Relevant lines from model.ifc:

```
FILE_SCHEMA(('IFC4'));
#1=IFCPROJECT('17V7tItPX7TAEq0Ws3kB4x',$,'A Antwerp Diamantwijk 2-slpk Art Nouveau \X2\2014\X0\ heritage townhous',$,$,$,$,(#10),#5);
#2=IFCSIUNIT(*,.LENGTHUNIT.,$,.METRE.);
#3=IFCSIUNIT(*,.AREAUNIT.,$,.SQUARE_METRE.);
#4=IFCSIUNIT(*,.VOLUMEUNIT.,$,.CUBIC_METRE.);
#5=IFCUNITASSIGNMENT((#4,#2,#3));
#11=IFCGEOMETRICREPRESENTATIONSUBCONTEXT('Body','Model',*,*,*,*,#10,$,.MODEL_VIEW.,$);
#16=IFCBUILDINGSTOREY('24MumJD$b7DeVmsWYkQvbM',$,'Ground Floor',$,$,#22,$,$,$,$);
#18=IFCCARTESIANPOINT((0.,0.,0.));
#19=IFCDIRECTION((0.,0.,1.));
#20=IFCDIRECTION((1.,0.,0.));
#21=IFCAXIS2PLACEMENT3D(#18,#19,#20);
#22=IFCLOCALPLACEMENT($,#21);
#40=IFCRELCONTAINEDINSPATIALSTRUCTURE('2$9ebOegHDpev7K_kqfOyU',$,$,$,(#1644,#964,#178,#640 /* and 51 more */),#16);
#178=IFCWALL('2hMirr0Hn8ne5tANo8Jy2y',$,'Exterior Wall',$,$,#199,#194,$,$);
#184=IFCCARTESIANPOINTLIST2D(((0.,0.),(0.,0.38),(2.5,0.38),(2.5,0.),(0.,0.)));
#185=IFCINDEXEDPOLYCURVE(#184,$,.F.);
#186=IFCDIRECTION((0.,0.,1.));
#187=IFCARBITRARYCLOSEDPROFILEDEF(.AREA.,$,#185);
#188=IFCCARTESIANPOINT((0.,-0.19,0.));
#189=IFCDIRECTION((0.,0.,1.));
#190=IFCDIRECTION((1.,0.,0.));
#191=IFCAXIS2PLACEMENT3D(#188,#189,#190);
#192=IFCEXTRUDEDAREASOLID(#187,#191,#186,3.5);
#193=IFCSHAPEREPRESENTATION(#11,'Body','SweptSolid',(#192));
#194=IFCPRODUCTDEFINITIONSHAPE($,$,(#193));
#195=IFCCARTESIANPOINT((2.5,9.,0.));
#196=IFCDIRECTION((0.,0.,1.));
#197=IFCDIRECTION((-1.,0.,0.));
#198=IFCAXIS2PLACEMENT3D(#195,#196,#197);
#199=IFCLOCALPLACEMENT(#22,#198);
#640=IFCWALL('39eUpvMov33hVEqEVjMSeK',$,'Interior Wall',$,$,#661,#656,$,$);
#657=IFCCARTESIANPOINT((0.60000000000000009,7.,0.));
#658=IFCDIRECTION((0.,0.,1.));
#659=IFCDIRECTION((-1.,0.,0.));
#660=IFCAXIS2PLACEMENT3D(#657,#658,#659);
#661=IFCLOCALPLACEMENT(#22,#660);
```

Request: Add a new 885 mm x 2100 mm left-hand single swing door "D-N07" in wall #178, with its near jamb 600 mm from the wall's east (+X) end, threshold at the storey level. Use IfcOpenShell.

```python
import numpy as np
import ifcopenshell
import ifcopenshell.api.feature
import ifcopenshell.api.geometry
import ifcopenshell.api.root
import ifcopenshell.api.spatial
import ifcopenshell.geom
import ifcopenshell.util.element
import ifcopenshell.util.placement
import ifcopenshell.util.representation
import ifcopenshell.util.shape
import ifcopenshell.util.unit

model = ifcopenshell.open("model.ifc")
unit_scale = ifcopenshell.util.unit.calculate_unit_scale(model)
settings = ifcopenshell.geom.settings()


def volume(element):
    """Net volume in cubic metres, openings subtracted."""
    shape = ifcopenshell.geom.create_shape(settings, element)
    return ifcopenshell.util.shape.get_volume(shape.geometry)


wall = model.by_guid("2hMirr0Hn8ne5tANo8Jy2y")
storey = ifcopenshell.util.element.get_container(wall, ifc_class="IfcBuildingStorey")
context = ifcopenshell.util.representation.get_context(model, "Model", "Body", "MODEL_VIEW")
before = volume(wall)

width, height, from_end, sill = 0.885, 2.1, 0.6, 0.0  # metres

# The wall runs along its own X axis, and the end named is its -X end.
wall_shape = ifcopenshell.geom.create_shape(settings, wall)
x, y, z = ifcopenshell.util.shape.get_vertices(wall_shape.geometry).T
start = x.min() + from_end
face, thickness = float(y.min()), float(y.max() - y.min())
wall_matrix = ifcopenshell.util.placement.get_local_placement(wall.ObjectPlacement)
level = ifcopenshell.util.placement.get_local_placement(storey.ObjectPlacement)[2, 3]


def in_wall(x, y):
    """Placement at x, y metres in the wall's axes, at sill height."""
    matrix = wall_matrix.copy()
    matrix[:, 3] = wall_matrix @ np.array([x / unit_scale, y / unit_scale, 0.0, 1.0])
    matrix[2, 3] = level + sill / unit_scale
    return matrix


# Opening: a box that overshoots both wall faces by 50 mm.
opening = ifcopenshell.api.root.create_entity(model, ifc_class="IfcOpeningElement", predefined_type="OPENING")
box = ifcopenshell.api.geometry.add_wall_representation(
    model, context=context, length=width, height=height, thickness=thickness + 0.1
)
ifcopenshell.api.geometry.assign_representation(model, product=opening, representation=box)
ifcopenshell.api.geometry.edit_object_placement(model, product=opening, matrix=in_wall(start, face - 0.05), is_si=False)
ifcopenshell.api.feature.add_feature(model, feature=opening, element=wall)

door = ifcopenshell.api.root.create_entity(model, ifc_class="IfcDoor", name="D-N07", predefined_type="DOOR")
door.OverallWidth, door.OverallHeight = width / unit_scale, height / unit_scale
door.OperationType = "SINGLE_SWING_LEFT"
body = ifcopenshell.api.geometry.add_door_representation(
    model,
    context=context,
    overall_width=door.OverallWidth,
    overall_height=door.OverallHeight,
    operation_type="SINGLE_SWING_LEFT",
    lining_properties={"LiningDepth": thickness / unit_scale, "ThresholdDepth": thickness / unit_scale},
)
ifcopenshell.api.geometry.assign_representation(model, product=door, representation=body)
ifcopenshell.api.spatial.assign_container(model, products=[door], relating_structure=storey)
ifcopenshell.api.feature.add_filling(model, opening=opening, element=door)

# The lining spans the wall, so the door starts at the wall face.
ifcopenshell.api.geometry.edit_object_placement(model, product=door, matrix=in_wall(start, face), is_si=False)

after = volume(wall)

print(f"wall volume {before:.3f} -> {after:.3f} m3")

model.write("model_edited.ifc")
```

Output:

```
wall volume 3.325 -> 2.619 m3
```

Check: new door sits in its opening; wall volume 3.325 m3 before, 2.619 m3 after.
